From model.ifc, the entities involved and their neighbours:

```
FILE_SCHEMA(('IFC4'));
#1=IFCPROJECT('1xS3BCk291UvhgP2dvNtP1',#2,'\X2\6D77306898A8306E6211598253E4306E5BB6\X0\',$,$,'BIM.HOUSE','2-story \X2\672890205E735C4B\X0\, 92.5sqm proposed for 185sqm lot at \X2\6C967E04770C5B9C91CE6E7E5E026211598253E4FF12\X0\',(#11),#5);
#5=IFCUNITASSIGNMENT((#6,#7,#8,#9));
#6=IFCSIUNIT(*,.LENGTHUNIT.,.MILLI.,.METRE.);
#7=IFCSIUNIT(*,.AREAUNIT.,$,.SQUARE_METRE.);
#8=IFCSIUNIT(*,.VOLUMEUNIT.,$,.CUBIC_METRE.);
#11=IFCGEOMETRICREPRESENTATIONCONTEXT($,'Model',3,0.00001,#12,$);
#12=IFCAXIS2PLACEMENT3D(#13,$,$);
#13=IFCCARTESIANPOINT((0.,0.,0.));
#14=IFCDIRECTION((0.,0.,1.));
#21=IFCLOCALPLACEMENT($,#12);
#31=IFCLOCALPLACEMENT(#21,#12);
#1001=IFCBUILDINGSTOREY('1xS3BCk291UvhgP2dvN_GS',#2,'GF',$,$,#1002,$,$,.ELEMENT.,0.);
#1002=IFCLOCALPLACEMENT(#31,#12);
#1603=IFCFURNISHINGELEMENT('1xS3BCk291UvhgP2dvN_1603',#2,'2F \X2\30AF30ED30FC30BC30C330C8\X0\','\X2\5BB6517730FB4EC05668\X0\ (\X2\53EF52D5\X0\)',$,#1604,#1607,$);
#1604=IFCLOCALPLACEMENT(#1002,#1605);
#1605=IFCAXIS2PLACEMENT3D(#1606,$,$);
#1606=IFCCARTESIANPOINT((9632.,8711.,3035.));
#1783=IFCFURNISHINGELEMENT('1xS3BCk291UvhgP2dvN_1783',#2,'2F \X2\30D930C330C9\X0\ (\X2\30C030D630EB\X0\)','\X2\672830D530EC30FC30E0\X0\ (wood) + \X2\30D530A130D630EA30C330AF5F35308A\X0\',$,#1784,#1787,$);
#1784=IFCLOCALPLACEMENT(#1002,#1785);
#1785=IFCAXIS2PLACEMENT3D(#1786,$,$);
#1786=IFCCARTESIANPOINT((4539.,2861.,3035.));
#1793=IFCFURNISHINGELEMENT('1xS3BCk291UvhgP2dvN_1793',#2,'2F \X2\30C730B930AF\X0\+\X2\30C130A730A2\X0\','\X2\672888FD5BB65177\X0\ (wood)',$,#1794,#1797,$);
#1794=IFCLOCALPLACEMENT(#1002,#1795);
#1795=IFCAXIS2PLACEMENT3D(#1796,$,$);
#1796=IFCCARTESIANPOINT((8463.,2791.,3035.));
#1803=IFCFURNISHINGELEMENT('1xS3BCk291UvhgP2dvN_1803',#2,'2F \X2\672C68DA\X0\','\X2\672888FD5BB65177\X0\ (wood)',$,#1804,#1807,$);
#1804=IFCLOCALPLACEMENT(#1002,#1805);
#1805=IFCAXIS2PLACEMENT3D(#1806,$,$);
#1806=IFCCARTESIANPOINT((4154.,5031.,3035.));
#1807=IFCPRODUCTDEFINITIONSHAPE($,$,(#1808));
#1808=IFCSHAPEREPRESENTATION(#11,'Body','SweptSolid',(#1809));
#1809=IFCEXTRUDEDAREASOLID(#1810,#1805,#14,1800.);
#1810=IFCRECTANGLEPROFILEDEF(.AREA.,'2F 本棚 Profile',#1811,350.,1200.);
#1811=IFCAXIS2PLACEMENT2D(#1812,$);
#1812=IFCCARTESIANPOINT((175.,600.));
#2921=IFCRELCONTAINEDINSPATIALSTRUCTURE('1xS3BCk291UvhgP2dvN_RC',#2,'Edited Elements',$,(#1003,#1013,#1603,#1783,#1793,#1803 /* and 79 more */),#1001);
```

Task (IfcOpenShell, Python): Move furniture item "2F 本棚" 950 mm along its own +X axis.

```python
import ifcopenshell
import ifcopenshell.api.geometry
import ifcopenshell.util.placement
import ifcopenshell.util.unit

model = ifcopenshell.open("model.ifc")
unit_scale = ifcopenshell.util.unit.calculate_unit_scale(model)

item = model.by_guid("1xS3BCk291UvhgP2dvN_1803")
matrix = ifcopenshell.util.placement.get_local_placement(item.ObjectPlacement)
matrix[:3, 3] += matrix[:3, 0] * 0.95 / unit_scale
ifcopenshell.api.geometry.edit_object_placement(model, product=item, matrix=matrix, is_si=False)

print(ifcopenshell.util.placement.get_local_placement(item.ObjectPlacement).round(3) + 0.0)

model.write("model_edited.ifc")
```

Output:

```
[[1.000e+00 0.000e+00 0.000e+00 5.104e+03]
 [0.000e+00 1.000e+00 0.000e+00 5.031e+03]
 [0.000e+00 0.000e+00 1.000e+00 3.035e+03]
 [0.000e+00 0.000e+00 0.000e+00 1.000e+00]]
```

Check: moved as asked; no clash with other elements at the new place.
